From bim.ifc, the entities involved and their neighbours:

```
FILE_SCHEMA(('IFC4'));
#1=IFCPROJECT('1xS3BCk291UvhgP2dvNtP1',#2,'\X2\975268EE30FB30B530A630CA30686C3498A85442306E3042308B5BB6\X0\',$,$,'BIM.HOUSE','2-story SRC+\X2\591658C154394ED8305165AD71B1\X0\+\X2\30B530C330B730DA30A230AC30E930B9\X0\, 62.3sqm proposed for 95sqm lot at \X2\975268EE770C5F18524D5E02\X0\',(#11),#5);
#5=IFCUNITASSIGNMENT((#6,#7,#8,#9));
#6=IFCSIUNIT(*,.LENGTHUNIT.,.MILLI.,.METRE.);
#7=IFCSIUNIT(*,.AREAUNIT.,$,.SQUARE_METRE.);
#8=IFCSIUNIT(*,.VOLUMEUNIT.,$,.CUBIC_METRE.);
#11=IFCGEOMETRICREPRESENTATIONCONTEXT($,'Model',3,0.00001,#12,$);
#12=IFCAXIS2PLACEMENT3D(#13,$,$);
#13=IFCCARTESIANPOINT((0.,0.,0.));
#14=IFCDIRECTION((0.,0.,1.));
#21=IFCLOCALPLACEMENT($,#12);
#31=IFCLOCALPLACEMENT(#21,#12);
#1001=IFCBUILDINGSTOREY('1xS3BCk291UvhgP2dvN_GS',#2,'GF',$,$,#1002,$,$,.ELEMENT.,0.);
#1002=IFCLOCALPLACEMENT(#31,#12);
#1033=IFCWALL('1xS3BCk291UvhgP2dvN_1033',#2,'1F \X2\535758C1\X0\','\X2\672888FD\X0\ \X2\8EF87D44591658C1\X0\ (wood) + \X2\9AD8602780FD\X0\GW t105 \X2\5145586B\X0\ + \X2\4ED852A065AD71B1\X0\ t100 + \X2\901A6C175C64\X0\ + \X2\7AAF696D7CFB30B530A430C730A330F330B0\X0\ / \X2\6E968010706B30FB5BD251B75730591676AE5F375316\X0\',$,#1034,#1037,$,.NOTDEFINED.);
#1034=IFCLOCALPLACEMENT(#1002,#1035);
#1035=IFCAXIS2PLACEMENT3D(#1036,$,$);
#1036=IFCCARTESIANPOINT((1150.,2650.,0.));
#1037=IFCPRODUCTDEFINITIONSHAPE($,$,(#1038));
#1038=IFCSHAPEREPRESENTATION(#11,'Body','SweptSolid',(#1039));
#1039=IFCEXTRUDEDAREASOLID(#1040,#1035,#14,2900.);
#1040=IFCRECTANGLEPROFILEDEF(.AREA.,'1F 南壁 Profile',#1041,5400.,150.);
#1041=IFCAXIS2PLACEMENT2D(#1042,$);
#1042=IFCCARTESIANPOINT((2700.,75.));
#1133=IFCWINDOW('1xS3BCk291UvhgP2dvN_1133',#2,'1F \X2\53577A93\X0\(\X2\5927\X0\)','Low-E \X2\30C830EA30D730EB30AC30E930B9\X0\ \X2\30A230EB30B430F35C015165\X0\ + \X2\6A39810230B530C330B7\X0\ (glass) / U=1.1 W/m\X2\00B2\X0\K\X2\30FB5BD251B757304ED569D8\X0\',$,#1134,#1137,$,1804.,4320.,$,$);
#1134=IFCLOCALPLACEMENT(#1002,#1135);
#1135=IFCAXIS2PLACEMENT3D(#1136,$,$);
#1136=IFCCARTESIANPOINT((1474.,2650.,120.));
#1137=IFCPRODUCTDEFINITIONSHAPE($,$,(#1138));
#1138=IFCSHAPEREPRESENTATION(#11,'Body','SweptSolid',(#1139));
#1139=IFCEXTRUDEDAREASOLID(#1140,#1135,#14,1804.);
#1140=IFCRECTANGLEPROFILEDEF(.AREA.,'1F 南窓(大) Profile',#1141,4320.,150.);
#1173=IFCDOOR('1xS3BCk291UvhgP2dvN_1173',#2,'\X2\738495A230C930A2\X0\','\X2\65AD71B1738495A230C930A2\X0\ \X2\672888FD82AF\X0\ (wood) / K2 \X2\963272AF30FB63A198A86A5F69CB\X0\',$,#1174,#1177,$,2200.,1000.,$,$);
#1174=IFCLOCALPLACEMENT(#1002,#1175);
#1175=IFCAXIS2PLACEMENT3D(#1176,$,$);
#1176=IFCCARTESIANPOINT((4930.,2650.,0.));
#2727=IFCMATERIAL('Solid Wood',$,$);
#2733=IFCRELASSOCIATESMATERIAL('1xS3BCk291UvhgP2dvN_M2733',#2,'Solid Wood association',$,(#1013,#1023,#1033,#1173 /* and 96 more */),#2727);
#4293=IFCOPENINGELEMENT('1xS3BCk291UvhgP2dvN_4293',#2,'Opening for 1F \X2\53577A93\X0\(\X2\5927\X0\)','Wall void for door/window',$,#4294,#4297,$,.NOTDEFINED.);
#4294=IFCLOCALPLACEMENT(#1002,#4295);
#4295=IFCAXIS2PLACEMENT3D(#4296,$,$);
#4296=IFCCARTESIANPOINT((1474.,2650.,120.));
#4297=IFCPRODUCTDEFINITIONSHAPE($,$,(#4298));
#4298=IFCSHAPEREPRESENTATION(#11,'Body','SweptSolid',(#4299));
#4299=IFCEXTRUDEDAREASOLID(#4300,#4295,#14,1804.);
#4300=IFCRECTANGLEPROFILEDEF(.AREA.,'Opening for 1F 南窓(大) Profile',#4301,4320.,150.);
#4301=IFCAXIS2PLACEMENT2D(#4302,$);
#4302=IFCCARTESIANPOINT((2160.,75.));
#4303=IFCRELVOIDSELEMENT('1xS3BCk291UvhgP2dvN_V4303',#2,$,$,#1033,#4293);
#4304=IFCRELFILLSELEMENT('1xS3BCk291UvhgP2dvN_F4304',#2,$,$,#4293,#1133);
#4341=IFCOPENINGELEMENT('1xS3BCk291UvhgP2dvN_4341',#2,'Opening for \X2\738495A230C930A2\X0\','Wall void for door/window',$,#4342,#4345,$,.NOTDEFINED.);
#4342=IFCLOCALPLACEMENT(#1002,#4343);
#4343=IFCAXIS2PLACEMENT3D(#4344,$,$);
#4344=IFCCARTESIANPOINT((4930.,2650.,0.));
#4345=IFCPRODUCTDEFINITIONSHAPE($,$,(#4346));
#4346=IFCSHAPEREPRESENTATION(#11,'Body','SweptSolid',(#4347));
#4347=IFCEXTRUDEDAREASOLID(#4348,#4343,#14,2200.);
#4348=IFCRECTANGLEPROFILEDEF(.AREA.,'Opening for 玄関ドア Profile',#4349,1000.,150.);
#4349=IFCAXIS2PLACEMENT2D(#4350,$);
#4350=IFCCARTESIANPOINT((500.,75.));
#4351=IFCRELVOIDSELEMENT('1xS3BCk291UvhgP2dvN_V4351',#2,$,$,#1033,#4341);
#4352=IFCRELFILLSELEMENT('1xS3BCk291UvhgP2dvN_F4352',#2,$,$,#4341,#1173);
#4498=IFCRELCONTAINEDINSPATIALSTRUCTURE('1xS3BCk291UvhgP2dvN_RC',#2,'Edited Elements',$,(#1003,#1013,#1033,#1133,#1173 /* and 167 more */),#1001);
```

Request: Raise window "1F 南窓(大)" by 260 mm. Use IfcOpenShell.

```python
import numpy as np
import ifcopenshell
import ifcopenshell.api.geometry
import ifcopenshell.util.placement
import ifcopenshell.util.unit

model = ifcopenshell.open("bim.ifc")
unit_scale = ifcopenshell.util.unit.calculate_unit_scale(model)

window = model.by_guid("1xS3BCk291UvhgP2dvN_1133")
opening = window.FillsVoids[0].RelatingOpeningElement
dz = 0.26 / unit_scale

shift = np.array([0.0, 0.0, dz])
# The window is not placed relative to its opening, so move both.
for product in (opening, window):
    matrix = ifcopenshell.util.placement.get_local_placement(product.ObjectPlacement)
    matrix[:3, 3] += shift
    ifcopenshell.api.geometry.edit_object_placement(model, product=product, matrix=matrix, is_si=False)

print(f"moved by {dz * unit_scale:+.3f} m")

model.write("bim_v2.ifc")
```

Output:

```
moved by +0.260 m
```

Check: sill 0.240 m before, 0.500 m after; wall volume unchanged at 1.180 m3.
